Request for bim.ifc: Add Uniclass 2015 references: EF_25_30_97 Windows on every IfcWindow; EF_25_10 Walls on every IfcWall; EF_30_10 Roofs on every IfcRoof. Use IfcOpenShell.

First a look at what the model holds.

```python
import ifcopenshell

model = ifcopenshell.open("bim.ifc")
print(model.schema)
print("classifications:", [c.Name for c in model.by_type("IfcClassification")])
for ifc_class in ("IfcDoor", "IfcRoof", "IfcStair", "IfcWall", "IfcWindow"):
    print(ifc_class, len(model.by_type(ifc_class)))
```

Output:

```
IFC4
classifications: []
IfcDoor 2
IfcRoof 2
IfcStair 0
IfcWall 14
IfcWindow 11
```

```python
import ifcopenshell
import ifcopenshell.api.classification

model = ifcopenshell.open("bim.ifc")

system = ifcopenshell.api.classification.add_classification(model, classification="Uniclass 2015")

codes = {
    "IfcWindow": ("EF_25_30_97", "Windows"),
    "IfcWall": ("EF_25_10", "Walls"),
    "IfcRoof": ("EF_30_10", "Roofs"),
}
for ifc_class, (code, name) in codes.items():
    products = model.by_type(ifc_class)
    ifcopenshell.api.classification.add_reference(
        model, products=products, classification=system, identification=code, name=name
    )
    print(code, len(products))

model.write("bim_v2.ifc")
```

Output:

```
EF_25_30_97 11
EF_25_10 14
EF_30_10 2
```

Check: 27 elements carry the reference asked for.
